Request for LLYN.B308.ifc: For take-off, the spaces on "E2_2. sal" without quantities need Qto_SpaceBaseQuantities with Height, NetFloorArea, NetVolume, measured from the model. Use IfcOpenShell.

First a look at what the model holds.

```python
import ifcopenshell
import ifcopenshell.util.element
import ifcopenshell.util.unit

model = ifcopenshell.open("LLYN.B308.ifc")
print(model.schema)
for unit_type in ("LENGTHUNIT", "AREAUNIT", "VOLUMEUNIT"):
    print(unit_type, ifcopenshell.util.unit.calculate_unit_scale(model, unit_type))
storey = next(s for s in model.by_type("IfcBuildingStorey") if s.Name == "E2_2. sal")
spaces = [e for e in ifcopenshell.util.element.get_decomposition(storey) if e.is_a("IfcSpace")]
for e in sorted(spaces, key=lambda e: e.id()):
    print(e.id(), e.is_a(), e.Name, list(ifcopenshell.util.element.get_psets(e, qtos_only=True)), sep=" | ")
```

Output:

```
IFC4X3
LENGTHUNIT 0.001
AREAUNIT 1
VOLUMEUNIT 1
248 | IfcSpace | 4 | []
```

```python
import ifcopenshell
import ifcopenshell.api.pset
import ifcopenshell.geom
import ifcopenshell.util.element
import ifcopenshell.util.shape
import ifcopenshell.util.unit

model = ifcopenshell.open("LLYN.B308.ifc")
unit_scale = ifcopenshell.util.unit.calculate_unit_scale(model)
area_scale = ifcopenshell.util.unit.calculate_unit_scale(model, "AREAUNIT")
volume_scale = ifcopenshell.util.unit.calculate_unit_scale(model, "VOLUMEUNIT")
settings = ifcopenshell.geom.settings()

storey = next(s for s in model.by_type("IfcBuildingStorey") if s.Name == "E2_2. sal")
spaces = [e for e in ifcopenshell.util.element.get_decomposition(storey) if e.is_a("IfcSpace")]

for e in sorted(spaces, key=lambda e: e.id()):
    if ifcopenshell.util.element.get_psets(e, qtos_only=True, should_inherit=False):
        continue
    # Geometry comes back in metres, in the element's own axes.
    shape = ifcopenshell.geom.create_shape(settings, e)
    values = {
        "Height": ifcopenshell.util.shape.get_z(shape.geometry) / unit_scale,
        "NetFloorArea": ifcopenshell.util.shape.get_footprint_area(shape.geometry) / area_scale,
        "NetVolume": ifcopenshell.util.shape.get_volume(shape.geometry) / volume_scale,
    }
    qto = ifcopenshell.api.pset.add_qto(model, product=e, name="Qto_SpaceBaseQuantities")
    ifcopenshell.api.pset.edit_qto(model, qto=qto, properties=values)
    print(e.id(), {k: round(v, 3) for k, v in values.items()})

model.write("LLYN.B308_v2.ifc")
```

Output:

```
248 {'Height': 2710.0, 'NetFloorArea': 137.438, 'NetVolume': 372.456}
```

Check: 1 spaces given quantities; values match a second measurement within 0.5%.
